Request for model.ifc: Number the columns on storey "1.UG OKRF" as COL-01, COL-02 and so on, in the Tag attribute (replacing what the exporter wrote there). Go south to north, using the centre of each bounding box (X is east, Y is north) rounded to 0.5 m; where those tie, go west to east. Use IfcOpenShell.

First a look at what the model holds.

```python
import ifcopenshell
import ifcopenshell.util.element
import ifcopenshell.util.placement

model = ifcopenshell.open("model.ifc")
print(model.schema)
storey = next(s for s in model.by_type("IfcBuildingStorey") if s.Name == "1.UG OKRF")
columns = [e for e in ifcopenshell.util.element.get_decomposition(storey) if e.is_a("IfcColumn")]
for e in sorted(columns, key=lambda e: e.id()):
    origin = ifcopenshell.util.placement.get_local_placement(e.ObjectPlacement)[:3, 3]
    print(e.id(), e.Tag, e.Name, origin.round(2) + 0.0, sep=" | ")
```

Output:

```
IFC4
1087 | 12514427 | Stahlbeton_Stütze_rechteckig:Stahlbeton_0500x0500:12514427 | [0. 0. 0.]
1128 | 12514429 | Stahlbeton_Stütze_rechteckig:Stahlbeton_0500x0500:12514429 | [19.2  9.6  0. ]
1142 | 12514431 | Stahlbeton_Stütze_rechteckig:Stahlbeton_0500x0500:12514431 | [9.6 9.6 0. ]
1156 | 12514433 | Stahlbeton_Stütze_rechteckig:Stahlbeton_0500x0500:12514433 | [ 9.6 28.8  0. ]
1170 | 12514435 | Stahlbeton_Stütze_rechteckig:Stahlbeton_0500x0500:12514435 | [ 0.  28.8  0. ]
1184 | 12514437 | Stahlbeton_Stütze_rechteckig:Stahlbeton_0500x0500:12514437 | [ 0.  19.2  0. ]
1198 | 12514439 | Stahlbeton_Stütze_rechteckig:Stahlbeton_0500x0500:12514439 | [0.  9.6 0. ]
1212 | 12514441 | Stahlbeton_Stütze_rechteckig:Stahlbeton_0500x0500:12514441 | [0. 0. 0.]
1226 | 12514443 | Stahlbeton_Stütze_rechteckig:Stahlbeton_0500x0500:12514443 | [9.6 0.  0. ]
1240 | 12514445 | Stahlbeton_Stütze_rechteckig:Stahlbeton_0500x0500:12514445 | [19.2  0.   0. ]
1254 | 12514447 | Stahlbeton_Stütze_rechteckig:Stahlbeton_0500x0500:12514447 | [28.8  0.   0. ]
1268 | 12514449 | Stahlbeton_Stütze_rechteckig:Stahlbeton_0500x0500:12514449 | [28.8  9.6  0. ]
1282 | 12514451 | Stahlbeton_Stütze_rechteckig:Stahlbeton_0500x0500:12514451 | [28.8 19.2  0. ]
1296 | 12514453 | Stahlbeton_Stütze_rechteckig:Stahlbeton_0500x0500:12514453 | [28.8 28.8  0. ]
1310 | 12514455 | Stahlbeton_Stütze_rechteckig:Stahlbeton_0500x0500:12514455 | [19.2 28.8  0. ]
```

```python
import ifcopenshell
import ifcopenshell.geom
import ifcopenshell.util.element
import ifcopenshell.util.shape

model = ifcopenshell.open("model.ifc")
settings = ifcopenshell.geom.settings()
settings.set("use-world-coords", True)


def centre(element):
    shape = ifcopenshell.geom.create_shape(settings, element)
    return ifcopenshell.util.shape.get_bbox_centroid(shape.geometry)


storey = next(s for s in model.by_type("IfcBuildingStorey") if s.Name == "1.UG OKRF")
columns = [e for e in ifcopenshell.util.element.get_decomposition(storey) if e.is_a("IfcColumn")]

# Insertion points can sit at a corner or the storey origin, so sort by the geometry (in metres).
centres = {e: centre(e) for e in columns}
columns.sort(key=lambda e: (round(centres[e][1] / 0.5), centres[e][0]))

for i, e in enumerate(columns, start=1):
    number = f"COL-{i:02d}"
    e.Tag = number
    print(e.id(), number)

model.write("model_v2.ifc")
```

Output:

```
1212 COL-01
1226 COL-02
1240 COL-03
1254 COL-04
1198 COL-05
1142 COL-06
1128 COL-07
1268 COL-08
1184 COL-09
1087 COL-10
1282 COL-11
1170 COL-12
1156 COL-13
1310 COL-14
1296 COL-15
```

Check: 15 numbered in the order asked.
